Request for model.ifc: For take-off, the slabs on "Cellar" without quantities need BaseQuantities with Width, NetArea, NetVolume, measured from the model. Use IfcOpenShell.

First a look at what the model holds.

```python
import ifcopenshell
import ifcopenshell.util.element
import ifcopenshell.util.unit

model = ifcopenshell.open("model.ifc")
print(model.schema)
for unit_type in ("LENGTHUNIT", "AREAUNIT", "VOLUMEUNIT"):
    print(unit_type, ifcopenshell.util.unit.calculate_unit_scale(model, unit_type))
storey = next(s for s in model.by_type("IfcBuildingStorey") if s.Name == "Cellar")
slabs = [e for e in ifcopenshell.util.element.get_decomposition(storey) if e.is_a("IfcSlab")]
for e in sorted(slabs, key=lambda e: e.id()):
    print(e.id(), e.is_a(), e.Name, list(ifcopenshell.util.element.get_psets(e, qtos_only=True)), sep=" | ")
```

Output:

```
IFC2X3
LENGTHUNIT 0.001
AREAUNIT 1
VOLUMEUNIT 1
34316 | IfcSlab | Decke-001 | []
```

```python
import ifcopenshell
import ifcopenshell.api.pset
import ifcopenshell.geom
import ifcopenshell.util.element
import ifcopenshell.util.shape
import ifcopenshell.util.unit

model = ifcopenshell.open("model.ifc")
unit_scale = ifcopenshell.util.unit.calculate_unit_scale(model)
area_scale = ifcopenshell.util.unit.calculate_unit_scale(model, "AREAUNIT")
volume_scale = ifcopenshell.util.unit.calculate_unit_scale(model, "VOLUMEUNIT")
settings = ifcopenshell.geom.settings()

storey = next(s for s in model.by_type("IfcBuildingStorey") if s.Name == "Cellar")
slabs = [e for e in ifcopenshell.util.element.get_decomposition(storey) if e.is_a("IfcSlab")]

for e in sorted(slabs, key=lambda e: e.id()):
    if ifcopenshell.util.element.get_psets(e, qtos_only=True, should_inherit=False):
        continue
    # Geometry comes back in metres, in the element's own axes.
    shape = ifcopenshell.geom.create_shape(settings, e)
    values = {
        "Width": ifcopenshell.util.shape.get_z(shape.geometry) / unit_scale,
        "NetArea": ifcopenshell.util.shape.get_footprint_area(shape.geometry) / area_scale,
        "NetVolume": ifcopenshell.util.shape.get_volume(shape.geometry) / volume_scale,
    }
    qto = ifcopenshell.api.pset.add_qto(model, product=e, name="BaseQuantities")
    ifcopenshell.api.pset.edit_qto(model, qto=qto, properties=values)
    print(e.id(), {k: round(v, 3) for k, v in values.items()})

model.write("model-out.ifc")
```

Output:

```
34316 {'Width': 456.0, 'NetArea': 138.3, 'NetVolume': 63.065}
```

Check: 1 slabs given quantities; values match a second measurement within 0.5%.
